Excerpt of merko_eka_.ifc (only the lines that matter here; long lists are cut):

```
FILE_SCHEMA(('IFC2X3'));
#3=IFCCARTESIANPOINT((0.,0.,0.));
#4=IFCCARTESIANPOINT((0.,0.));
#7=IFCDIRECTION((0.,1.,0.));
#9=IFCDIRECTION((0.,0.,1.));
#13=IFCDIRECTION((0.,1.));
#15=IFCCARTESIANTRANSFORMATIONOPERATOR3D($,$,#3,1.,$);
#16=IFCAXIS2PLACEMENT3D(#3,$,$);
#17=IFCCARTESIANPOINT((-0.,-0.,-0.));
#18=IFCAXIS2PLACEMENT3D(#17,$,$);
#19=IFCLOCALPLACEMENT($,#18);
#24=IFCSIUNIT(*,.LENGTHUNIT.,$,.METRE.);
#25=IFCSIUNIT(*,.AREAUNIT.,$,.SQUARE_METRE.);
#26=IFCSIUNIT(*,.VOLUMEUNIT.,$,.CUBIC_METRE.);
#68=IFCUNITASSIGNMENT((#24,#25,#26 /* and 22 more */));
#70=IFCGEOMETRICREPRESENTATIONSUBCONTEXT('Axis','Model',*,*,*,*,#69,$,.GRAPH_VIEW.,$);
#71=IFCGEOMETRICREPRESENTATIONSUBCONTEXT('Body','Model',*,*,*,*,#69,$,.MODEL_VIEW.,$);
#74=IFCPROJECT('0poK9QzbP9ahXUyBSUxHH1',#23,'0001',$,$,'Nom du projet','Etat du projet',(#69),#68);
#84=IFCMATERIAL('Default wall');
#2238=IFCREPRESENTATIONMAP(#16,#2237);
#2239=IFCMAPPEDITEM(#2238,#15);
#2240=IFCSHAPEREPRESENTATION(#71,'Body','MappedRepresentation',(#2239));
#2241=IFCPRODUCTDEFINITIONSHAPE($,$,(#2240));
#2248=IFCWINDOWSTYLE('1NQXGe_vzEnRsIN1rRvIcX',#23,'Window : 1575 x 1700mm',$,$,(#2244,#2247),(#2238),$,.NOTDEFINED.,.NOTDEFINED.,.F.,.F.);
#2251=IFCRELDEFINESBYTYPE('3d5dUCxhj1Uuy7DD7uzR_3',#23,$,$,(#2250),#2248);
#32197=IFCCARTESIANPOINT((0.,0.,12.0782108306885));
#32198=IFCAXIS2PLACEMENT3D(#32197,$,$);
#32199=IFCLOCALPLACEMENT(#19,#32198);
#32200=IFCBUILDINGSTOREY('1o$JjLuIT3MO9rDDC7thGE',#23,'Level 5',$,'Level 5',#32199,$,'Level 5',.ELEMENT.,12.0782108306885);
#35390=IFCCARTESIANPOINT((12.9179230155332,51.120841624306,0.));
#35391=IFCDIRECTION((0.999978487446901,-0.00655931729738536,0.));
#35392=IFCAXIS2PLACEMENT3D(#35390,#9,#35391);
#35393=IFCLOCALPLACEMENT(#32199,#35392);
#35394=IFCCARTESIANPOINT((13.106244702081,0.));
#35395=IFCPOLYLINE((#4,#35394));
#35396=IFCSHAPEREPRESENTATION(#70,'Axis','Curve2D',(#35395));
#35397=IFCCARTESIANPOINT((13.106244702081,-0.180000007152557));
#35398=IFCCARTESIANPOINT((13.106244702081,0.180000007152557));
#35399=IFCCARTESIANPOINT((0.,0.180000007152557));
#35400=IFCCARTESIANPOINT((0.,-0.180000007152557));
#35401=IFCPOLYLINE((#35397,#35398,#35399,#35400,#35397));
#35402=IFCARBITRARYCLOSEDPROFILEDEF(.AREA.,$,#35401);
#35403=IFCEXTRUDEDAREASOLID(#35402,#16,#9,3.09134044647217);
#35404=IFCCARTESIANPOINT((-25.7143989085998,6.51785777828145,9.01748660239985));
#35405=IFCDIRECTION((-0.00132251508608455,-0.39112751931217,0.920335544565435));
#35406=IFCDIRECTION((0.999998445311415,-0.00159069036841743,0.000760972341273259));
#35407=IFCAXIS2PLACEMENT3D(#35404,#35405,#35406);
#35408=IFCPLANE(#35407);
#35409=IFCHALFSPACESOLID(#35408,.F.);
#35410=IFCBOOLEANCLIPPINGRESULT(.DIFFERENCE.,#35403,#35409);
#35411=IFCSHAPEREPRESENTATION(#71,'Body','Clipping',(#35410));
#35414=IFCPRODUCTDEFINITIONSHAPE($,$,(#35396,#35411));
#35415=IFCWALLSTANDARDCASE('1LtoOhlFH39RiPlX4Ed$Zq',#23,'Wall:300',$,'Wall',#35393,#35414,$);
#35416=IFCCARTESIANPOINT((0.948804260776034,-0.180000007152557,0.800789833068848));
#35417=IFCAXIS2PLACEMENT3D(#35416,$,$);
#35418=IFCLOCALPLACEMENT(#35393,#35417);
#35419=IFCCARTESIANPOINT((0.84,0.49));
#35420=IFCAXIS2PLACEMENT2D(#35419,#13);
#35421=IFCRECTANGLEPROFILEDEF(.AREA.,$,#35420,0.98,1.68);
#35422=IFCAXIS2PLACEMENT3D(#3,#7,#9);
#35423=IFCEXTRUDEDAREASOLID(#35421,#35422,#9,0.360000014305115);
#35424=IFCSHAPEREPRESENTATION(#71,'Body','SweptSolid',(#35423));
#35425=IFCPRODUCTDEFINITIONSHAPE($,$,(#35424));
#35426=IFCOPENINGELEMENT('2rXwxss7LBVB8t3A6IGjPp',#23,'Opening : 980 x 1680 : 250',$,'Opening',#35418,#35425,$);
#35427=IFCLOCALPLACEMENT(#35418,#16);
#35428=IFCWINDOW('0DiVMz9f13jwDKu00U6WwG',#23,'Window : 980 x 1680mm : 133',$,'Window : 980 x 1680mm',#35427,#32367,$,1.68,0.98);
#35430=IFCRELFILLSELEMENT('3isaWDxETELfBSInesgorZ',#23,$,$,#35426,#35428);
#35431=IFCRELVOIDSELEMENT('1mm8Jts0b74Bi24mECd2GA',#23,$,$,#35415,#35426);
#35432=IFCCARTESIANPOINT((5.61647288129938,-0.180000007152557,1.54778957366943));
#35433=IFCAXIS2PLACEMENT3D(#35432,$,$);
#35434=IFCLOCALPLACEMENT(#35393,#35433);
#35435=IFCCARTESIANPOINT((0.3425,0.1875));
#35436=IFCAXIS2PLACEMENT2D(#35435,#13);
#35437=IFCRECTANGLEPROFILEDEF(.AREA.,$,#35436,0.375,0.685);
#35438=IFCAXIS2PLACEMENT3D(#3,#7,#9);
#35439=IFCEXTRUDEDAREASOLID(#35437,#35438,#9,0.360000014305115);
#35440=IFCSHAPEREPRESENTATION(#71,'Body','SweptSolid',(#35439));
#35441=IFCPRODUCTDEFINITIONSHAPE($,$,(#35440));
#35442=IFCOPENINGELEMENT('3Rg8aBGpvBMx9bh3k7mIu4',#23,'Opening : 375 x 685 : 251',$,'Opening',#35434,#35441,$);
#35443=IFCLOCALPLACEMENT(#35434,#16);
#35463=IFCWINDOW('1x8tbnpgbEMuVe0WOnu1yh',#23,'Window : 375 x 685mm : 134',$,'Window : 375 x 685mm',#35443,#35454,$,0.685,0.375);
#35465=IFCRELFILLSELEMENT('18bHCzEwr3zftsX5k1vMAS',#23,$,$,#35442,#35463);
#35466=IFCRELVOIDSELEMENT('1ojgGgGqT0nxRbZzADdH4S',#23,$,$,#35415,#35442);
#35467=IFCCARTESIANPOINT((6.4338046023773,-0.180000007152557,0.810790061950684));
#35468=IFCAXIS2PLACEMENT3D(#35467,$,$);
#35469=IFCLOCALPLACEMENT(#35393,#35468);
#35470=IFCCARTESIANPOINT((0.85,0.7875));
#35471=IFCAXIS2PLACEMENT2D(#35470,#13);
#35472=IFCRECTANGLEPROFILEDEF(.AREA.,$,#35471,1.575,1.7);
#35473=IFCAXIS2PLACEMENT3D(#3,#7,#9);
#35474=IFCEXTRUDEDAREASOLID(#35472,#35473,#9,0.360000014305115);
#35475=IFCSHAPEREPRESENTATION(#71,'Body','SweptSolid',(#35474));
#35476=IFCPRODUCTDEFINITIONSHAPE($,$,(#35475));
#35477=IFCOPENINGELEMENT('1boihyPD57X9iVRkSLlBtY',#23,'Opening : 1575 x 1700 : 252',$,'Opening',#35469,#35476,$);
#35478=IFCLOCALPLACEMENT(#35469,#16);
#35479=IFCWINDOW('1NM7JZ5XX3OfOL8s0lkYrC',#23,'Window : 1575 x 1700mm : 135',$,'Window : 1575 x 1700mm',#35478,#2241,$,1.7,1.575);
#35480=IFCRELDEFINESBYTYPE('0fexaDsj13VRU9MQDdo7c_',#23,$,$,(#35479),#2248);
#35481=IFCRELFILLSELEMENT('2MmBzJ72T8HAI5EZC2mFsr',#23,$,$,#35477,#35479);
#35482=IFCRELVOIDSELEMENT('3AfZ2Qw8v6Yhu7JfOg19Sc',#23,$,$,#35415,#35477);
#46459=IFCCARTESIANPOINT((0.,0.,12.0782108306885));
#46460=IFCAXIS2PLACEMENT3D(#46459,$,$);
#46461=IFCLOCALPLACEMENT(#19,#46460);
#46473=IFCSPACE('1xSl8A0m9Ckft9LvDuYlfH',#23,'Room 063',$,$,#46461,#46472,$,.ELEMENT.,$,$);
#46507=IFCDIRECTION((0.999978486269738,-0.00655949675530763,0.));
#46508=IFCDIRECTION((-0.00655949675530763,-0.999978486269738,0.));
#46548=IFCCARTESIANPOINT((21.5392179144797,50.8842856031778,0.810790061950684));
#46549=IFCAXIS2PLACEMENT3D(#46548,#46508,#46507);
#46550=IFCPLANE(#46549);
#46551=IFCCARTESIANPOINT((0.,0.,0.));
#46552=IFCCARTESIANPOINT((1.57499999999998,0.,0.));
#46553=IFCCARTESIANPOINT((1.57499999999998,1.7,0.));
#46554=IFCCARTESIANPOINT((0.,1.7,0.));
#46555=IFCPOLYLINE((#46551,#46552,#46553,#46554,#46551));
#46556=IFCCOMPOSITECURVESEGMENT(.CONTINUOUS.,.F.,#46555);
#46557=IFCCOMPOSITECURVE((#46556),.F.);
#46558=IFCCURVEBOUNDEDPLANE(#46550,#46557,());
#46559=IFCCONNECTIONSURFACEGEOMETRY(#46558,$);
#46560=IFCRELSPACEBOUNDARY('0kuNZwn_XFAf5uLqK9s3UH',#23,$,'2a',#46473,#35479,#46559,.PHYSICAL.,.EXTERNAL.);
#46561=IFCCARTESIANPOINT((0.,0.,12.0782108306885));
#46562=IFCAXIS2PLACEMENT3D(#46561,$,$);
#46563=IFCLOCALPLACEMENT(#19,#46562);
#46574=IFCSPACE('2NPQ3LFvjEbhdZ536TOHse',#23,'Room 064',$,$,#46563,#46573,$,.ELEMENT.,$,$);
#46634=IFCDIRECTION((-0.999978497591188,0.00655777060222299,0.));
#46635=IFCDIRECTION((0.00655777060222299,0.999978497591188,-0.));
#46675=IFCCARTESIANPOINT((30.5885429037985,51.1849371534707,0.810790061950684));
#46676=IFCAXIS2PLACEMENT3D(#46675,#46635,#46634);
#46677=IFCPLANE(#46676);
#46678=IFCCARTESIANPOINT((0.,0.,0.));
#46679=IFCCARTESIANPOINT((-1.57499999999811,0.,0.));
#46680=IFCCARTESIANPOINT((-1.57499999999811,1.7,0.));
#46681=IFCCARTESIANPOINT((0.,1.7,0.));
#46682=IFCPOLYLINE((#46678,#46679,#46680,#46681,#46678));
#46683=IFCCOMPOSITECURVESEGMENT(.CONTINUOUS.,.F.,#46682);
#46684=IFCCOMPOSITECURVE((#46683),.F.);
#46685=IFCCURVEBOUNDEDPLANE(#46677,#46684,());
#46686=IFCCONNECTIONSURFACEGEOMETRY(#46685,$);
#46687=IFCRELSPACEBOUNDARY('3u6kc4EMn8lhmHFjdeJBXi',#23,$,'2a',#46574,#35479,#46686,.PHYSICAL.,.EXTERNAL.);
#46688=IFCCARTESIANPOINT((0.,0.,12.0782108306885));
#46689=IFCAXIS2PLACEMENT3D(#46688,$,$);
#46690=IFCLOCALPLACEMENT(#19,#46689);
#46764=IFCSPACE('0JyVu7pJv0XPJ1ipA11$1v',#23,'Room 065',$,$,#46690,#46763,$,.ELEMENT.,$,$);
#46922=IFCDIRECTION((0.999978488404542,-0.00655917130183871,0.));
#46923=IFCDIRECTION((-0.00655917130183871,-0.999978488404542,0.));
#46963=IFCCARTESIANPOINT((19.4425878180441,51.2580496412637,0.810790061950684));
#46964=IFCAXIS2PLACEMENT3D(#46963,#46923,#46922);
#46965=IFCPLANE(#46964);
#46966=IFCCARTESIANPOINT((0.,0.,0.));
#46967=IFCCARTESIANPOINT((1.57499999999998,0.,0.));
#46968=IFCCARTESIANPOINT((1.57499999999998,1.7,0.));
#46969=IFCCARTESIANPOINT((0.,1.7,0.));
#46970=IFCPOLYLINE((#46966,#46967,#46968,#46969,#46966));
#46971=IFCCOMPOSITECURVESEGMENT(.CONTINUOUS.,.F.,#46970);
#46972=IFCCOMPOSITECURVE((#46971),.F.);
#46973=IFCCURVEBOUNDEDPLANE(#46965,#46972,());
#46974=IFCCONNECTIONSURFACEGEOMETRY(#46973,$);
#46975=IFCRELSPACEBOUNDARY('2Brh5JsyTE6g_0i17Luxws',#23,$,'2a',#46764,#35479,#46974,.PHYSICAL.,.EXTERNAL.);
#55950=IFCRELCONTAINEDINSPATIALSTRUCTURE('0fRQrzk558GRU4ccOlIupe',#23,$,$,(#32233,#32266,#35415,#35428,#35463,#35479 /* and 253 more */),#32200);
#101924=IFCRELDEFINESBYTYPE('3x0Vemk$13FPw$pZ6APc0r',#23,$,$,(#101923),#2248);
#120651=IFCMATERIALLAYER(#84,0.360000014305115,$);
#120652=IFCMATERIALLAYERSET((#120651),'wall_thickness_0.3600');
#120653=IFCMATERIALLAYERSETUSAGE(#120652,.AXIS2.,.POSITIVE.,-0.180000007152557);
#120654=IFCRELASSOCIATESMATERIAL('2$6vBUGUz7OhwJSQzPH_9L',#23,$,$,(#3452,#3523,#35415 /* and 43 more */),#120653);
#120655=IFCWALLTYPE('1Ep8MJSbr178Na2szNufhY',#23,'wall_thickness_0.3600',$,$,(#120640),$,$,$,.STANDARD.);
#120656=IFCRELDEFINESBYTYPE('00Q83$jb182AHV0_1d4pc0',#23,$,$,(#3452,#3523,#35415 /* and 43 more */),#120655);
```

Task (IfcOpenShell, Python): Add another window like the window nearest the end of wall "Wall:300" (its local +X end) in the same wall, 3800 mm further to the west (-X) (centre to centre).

```python
import numpy as np
import ifcopenshell
import ifcopenshell.api.feature
import ifcopenshell.api.geometry
import ifcopenshell.api.root
import ifcopenshell.geom
import ifcopenshell.util.element
import ifcopenshell.util.placement
import ifcopenshell.util.shape

model = ifcopenshell.open("merko_eka_.ifc")
settings = ifcopenshell.geom.settings()


def volume(element):
    """Net volume in cubic metres, openings subtracted."""
    shape = ifcopenshell.geom.create_shape(settings, element)
    return ifcopenshell.util.shape.get_volume(shape.geometry)


window = model.by_id(35479)
opening = window.FillsVoids[0].RelatingOpeningElement
wall = opening.VoidsElements[0].RelatingBuildingElement
before = volume(wall)
shift = ifcopenshell.util.placement.get_local_placement(wall.ObjectPlacement)[:3, 0] * -3.8

# copy_class copies the void relationship, type, container and properties, but no geometry.
new_opening = ifcopenshell.api.root.copy_class(model, product=opening)
new_opening.Representation = ifcopenshell.util.element.copy_deep(
    model, opening.Representation, exclude=["IfcGeometricRepresentationContext", "IfcRepresentationMap"]
)
new_opening.Name = "Opening : 1575 x 1700"
new_window = ifcopenshell.api.root.copy_class(model, product=window)
new_window.Representation = ifcopenshell.util.element.copy_deep(
    model, window.Representation, exclude=["IfcGeometricRepresentationContext", "IfcRepresentationMap"]
)
new_window.Name = "Window : 1575 x 1700mm"
fills = ifcopenshell.api.feature.add_filling(model, opening=new_opening, element=new_window)
fills.OwnerHistory = new_window.OwnerHistory  # required in IFC2X3

for old, new in ((opening, new_opening), (window, new_window)):
    matrix = ifcopenshell.util.placement.get_local_placement(old.ObjectPlacement)
    matrix[:3, 3] += shift
    ifcopenshell.api.geometry.edit_object_placement(model, product=new, matrix=matrix, is_si=False)

# The copied space boundaries still share their surfaces with the original.
for rel in new_window.ProvidesBoundaries:
    if rel.ConnectionGeometry:
        rel.ConnectionGeometry = ifcopenshell.util.element.copy_deep(model, rel.ConnectionGeometry)

# Space boundary surfaces are stored in each space's coordinates; move them too.
for rel in new_window.ProvidesBoundaries:
    if not rel.ConnectionGeometry:
        continue
    surface = rel.ConnectionGeometry.SurfaceOnRelatingElement.BasisSurface
    space_matrix = ifcopenshell.util.placement.get_local_placement(rel.RelatingSpace.ObjectPlacement)
    point = np.array(surface.Position.Location.Coordinates) + space_matrix[:3, :3].T @ shift
    surface.Position = model.createIfcAxis2Placement3D(
        model.createIfcCartesianPoint(point.tolist()), surface.Position.Axis, surface.Position.RefDirection
    )

after = volume(wall)

print(f"wall volume {before:.3f} -> {after:.3f} m3")

model.write("merko_eka__updated.ifc")
```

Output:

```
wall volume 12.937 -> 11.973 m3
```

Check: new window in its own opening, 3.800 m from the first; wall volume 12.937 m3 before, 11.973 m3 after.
